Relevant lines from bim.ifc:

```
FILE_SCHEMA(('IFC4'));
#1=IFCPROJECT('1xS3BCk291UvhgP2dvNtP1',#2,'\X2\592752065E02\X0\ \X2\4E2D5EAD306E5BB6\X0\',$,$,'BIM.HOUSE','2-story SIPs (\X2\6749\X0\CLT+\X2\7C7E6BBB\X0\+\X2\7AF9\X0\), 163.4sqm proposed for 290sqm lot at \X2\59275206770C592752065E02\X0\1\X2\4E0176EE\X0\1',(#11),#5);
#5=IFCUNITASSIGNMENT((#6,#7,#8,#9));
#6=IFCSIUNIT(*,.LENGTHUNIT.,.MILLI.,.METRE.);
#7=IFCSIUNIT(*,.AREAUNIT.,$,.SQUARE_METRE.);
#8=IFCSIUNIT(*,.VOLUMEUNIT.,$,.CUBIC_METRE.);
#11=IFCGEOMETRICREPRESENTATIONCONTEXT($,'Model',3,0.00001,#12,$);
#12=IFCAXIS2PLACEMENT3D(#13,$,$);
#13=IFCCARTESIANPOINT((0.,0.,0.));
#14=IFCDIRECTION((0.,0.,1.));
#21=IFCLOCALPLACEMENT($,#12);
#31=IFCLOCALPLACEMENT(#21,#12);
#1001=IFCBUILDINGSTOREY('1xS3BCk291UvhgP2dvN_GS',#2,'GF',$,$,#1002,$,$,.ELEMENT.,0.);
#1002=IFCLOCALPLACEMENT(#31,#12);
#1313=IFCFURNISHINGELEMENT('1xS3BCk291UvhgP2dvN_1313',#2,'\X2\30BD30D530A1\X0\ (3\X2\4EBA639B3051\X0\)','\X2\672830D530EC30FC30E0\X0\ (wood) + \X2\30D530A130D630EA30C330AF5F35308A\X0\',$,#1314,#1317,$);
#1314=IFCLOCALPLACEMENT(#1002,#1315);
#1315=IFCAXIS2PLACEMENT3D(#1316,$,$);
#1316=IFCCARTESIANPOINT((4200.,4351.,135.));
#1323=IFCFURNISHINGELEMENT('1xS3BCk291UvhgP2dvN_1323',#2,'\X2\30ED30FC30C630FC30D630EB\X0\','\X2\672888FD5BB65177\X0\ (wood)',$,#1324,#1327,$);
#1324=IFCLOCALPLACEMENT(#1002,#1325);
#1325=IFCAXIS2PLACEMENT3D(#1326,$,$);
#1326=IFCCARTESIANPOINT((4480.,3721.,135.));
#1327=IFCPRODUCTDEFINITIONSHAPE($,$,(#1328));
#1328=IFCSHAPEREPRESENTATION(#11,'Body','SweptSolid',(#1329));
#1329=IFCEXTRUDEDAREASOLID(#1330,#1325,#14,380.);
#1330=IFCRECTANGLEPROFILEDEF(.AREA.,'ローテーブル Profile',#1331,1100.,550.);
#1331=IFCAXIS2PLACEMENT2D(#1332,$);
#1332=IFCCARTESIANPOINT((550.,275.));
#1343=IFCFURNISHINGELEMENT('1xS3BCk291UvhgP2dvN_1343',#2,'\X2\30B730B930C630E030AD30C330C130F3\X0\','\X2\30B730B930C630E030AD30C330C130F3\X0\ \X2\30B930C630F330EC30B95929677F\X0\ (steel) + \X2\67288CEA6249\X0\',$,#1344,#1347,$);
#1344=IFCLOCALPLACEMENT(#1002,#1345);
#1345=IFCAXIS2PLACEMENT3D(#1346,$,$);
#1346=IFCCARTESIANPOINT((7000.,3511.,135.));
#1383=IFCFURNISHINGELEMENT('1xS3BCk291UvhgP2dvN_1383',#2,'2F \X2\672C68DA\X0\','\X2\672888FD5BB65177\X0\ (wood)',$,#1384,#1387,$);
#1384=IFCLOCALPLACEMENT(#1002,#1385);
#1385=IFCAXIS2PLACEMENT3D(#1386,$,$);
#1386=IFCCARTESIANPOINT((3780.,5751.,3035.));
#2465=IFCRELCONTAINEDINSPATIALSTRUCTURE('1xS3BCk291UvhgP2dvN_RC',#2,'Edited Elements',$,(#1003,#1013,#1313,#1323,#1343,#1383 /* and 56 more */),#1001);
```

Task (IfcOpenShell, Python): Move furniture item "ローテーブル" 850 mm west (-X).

```python
import ifcopenshell
import ifcopenshell.api.geometry
import ifcopenshell.util.placement
import ifcopenshell.util.unit

model = ifcopenshell.open("bim.ifc")
unit_scale = ifcopenshell.util.unit.calculate_unit_scale(model)

item = model.by_id(1323)
matrix = ifcopenshell.util.placement.get_local_placement(item.ObjectPlacement)
matrix[0, 3] -= 0.85 / unit_scale
ifcopenshell.api.geometry.edit_object_placement(model, product=item, matrix=matrix, is_si=False)

print(ifcopenshell.util.placement.get_local_placement(item.ObjectPlacement).round(3) + 0.0)

model.write("bim_updated.ifc")
```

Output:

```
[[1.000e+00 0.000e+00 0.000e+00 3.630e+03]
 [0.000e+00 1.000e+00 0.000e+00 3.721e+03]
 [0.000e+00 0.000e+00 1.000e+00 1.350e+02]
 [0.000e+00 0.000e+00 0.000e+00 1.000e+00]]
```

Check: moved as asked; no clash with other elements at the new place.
